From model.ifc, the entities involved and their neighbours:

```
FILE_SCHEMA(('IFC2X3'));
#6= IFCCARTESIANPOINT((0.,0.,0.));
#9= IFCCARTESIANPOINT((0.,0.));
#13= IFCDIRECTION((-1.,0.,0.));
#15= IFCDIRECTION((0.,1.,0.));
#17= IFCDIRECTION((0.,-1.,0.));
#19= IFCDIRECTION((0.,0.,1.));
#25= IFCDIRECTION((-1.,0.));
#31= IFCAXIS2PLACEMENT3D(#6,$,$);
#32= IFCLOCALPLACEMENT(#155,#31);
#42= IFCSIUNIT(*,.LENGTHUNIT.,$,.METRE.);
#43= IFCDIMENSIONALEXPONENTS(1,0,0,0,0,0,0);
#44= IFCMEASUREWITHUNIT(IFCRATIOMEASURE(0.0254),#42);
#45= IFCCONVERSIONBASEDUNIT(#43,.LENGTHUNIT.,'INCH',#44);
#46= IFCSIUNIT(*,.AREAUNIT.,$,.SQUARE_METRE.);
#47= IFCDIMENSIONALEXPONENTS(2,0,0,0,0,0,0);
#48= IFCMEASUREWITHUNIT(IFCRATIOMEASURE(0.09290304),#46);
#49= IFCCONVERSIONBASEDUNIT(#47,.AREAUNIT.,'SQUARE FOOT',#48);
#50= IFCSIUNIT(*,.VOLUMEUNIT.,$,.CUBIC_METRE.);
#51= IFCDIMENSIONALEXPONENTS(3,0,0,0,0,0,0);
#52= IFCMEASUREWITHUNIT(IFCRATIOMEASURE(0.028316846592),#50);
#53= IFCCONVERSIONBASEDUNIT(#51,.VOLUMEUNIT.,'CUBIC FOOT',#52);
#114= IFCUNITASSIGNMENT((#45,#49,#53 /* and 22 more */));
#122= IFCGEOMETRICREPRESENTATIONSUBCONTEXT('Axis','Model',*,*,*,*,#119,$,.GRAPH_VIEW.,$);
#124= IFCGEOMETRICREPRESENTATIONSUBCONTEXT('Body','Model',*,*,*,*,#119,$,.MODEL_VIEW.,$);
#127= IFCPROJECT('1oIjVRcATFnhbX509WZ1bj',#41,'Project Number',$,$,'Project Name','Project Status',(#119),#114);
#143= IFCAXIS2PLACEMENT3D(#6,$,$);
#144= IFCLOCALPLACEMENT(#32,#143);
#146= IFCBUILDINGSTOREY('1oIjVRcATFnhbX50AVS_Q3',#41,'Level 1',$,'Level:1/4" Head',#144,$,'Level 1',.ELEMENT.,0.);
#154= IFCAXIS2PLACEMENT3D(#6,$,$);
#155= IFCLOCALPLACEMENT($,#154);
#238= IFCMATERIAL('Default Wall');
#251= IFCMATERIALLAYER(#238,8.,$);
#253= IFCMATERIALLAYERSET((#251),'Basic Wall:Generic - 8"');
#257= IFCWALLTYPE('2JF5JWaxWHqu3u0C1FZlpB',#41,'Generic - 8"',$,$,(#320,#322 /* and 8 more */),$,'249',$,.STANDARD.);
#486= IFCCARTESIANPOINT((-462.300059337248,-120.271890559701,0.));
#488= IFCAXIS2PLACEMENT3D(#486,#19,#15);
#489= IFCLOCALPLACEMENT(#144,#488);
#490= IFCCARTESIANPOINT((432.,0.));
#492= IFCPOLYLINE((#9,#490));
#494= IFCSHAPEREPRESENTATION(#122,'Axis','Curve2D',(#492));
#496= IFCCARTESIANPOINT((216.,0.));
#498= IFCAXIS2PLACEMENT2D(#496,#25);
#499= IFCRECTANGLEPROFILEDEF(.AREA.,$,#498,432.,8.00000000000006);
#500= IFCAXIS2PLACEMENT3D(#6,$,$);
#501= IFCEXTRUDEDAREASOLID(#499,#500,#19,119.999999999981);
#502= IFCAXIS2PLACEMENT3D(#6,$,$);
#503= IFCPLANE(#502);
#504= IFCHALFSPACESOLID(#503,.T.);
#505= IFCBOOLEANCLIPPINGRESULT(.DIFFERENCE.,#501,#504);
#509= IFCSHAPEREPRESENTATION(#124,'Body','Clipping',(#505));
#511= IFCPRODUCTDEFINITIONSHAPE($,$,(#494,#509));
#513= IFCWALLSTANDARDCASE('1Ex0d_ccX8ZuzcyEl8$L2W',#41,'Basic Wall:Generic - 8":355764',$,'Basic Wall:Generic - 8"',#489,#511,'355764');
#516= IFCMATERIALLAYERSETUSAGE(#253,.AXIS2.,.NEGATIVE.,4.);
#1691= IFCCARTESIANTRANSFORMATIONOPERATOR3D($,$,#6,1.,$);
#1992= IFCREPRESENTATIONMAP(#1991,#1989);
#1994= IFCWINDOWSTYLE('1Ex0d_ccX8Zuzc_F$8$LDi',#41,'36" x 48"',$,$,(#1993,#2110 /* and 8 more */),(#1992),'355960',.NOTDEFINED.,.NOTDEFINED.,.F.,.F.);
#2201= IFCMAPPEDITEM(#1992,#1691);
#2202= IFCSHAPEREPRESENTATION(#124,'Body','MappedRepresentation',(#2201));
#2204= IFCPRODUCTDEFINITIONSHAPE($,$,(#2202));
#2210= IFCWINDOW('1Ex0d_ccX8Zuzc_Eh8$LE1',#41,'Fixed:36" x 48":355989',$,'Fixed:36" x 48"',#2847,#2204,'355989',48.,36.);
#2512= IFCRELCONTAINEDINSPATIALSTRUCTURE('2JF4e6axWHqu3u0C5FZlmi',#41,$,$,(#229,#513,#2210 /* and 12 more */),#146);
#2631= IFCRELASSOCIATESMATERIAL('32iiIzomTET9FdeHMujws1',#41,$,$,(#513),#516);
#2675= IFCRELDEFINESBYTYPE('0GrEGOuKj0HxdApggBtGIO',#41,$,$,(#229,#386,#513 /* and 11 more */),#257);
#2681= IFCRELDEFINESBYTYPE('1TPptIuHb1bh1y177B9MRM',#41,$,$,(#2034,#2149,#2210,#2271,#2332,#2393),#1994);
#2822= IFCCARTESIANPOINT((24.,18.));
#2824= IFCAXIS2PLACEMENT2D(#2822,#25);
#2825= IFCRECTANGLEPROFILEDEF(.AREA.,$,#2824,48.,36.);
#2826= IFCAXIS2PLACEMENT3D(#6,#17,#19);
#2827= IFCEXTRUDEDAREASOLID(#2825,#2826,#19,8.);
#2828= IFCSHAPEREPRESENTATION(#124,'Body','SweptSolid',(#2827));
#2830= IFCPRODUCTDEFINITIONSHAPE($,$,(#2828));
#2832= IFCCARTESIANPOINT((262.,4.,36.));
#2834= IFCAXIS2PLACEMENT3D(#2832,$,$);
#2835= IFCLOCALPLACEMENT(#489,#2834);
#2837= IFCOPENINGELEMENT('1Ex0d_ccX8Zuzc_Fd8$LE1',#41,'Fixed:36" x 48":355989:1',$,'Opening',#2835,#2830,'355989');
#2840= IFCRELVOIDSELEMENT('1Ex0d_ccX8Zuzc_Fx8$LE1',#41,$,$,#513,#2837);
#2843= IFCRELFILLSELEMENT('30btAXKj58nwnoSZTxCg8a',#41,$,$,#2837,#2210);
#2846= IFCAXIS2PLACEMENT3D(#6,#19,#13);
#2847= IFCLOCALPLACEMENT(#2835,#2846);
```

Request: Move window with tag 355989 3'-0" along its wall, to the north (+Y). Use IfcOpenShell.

```python
import ifcopenshell
import ifcopenshell.api.geometry
import ifcopenshell.util.placement
import ifcopenshell.util.unit

model = ifcopenshell.open("model.ifc")
unit_scale = ifcopenshell.util.unit.calculate_unit_scale(model)

window = model.by_guid("1Ex0d_ccX8Zuzc_Eh8$LE1")
opening = window.FillsVoids[0].RelatingOpeningElement
wall = opening.VoidsElements[0].RelatingBuildingElement

wall_matrix = ifcopenshell.util.placement.get_local_placement(wall.ObjectPlacement)
shift = wall_matrix[:3, 0] * 36 * 0.0254 / unit_scale
before = ifcopenshell.util.placement.get_local_placement(window.ObjectPlacement)[:3, 3].copy()

# The window is placed relative to its opening, so it follows when the opening moves.
matrix = ifcopenshell.util.placement.get_local_placement(opening.ObjectPlacement)
matrix[:3, 3] += shift
ifcopenshell.api.geometry.edit_object_placement(
    model, product=opening, matrix=matrix, is_si=False, should_transform_children=True
)

after = ifcopenshell.util.placement.get_local_placement(window.ObjectPlacement)[:3, 3]
print("window moved by", (after - before).round(3) + 0.0)

model.write("model_edited.ifc")
```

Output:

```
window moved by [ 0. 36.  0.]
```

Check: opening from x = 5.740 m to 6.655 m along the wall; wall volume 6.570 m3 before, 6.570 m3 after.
